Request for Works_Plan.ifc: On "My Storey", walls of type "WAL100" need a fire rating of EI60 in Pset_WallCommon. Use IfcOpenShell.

First a look at what the model holds.

```python
import ifcopenshell
import ifcopenshell.util.element

model = ifcopenshell.open("Works_Plan.ifc")
print(model.schema)
storey = next(s for s in model.by_type("IfcBuildingStorey") if s.Name == "My Storey")
walls = [e for e in ifcopenshell.util.element.get_decomposition(storey) if e.is_a("IfcWall")]
seen = {}
for e in walls:
    element_type = ifcopenshell.util.element.get_type(e)
    key = (element_type.Name if element_type != e and element_type else None, ifcopenshell.util.element.get_pset(e, "Pset_WallCommon", "FireRating"))
    seen[key] = seen.get(key, 0) + 1
for (name, value), count in sorted(seen.items(), key=str):
    print(count, "x", name, "|", value)
```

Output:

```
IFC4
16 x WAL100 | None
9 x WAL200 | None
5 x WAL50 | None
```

```python
import ifcopenshell
import ifcopenshell.api.pset
import ifcopenshell.util.element

model = ifcopenshell.open("Works_Plan.ifc")

storey = next(s for s in model.by_type("IfcBuildingStorey") if s.Name == "My Storey")
walls = [e for e in ifcopenshell.util.element.get_decomposition(storey) if e.is_a("IfcWall")]

count = 0
for e in walls:
    element_type = ifcopenshell.util.element.get_type(e)
    if element_type in (None, e) or element_type.Name != "WAL100":
        continue
    # add_pset returns the element's existing set when there is one.
    pset = ifcopenshell.api.pset.add_pset(model, product=e, name="Pset_WallCommon")
    ifcopenshell.api.pset.edit_pset(model, pset=pset, properties={"FireRating": "EI60"})
    count += 1

print(count, "walls updated")

model.write("Works_Plan_rev.ifc")
```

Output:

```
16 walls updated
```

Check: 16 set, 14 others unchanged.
